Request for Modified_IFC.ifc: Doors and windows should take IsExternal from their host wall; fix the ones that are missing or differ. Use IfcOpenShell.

First a look at what the model holds.

```python
import ifcopenshell
import ifcopenshell.util.element

model = ifcopenshell.open("Modified_IFC.ifc")
print(model.schema)
seen = {}
for e in model.by_type("IfcDoor") + model.by_type("IfcWindow"):
    if not e.FillsVoids:
        continue
    host = e.FillsVoids[0].RelatingOpeningElement.VoidsElements[0].RelatingBuildingElement
    own = ifcopenshell.util.element.get_pset(e, f"Pset_{e.is_a()[3:].removesuffix('StandardCase')}Common", "IsExternal")
    wall = ifcopenshell.util.element.get_pset(host, "Pset_WallCommon", "IsExternal")
    seen[e.is_a(), own, wall] = seen.get((e.is_a(), own, wall), 0) + 1
for (cls, own, wall), count in sorted(seen.items(), key=str):
    print(count, cls, "IsExternal:", own, "| host wall:", wall)
```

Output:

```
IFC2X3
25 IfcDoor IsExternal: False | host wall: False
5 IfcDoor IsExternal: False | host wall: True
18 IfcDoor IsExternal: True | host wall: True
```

```python
import ifcopenshell
import ifcopenshell.api.pset
import ifcopenshell.util.element

model = ifcopenshell.open("Modified_IFC.ifc")

count = 0
for ifc_class, pset_name in (("IfcDoor", "Pset_DoorCommon"), ("IfcWindow", "Pset_WindowCommon")):
    for e in model.by_type(ifc_class):
        if not e.FillsVoids:
            continue
        host = e.FillsVoids[0].RelatingOpeningElement.VoidsElements[0].RelatingBuildingElement
        external = ifcopenshell.util.element.get_pset(host, "Pset_WallCommon", "IsExternal")
        if external is None or ifcopenshell.util.element.get_pset(e, pset_name, "IsExternal") == external:
            continue
        pset = ifcopenshell.api.pset.add_pset(model, product=e, name=pset_name)
        ifcopenshell.api.pset.edit_pset(model, pset=pset, properties={"IsExternal": external})
        count += 1

print(count, "updated")

model.write("Modified_IFC_updated.ifc")
```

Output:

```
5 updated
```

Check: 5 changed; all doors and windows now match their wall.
